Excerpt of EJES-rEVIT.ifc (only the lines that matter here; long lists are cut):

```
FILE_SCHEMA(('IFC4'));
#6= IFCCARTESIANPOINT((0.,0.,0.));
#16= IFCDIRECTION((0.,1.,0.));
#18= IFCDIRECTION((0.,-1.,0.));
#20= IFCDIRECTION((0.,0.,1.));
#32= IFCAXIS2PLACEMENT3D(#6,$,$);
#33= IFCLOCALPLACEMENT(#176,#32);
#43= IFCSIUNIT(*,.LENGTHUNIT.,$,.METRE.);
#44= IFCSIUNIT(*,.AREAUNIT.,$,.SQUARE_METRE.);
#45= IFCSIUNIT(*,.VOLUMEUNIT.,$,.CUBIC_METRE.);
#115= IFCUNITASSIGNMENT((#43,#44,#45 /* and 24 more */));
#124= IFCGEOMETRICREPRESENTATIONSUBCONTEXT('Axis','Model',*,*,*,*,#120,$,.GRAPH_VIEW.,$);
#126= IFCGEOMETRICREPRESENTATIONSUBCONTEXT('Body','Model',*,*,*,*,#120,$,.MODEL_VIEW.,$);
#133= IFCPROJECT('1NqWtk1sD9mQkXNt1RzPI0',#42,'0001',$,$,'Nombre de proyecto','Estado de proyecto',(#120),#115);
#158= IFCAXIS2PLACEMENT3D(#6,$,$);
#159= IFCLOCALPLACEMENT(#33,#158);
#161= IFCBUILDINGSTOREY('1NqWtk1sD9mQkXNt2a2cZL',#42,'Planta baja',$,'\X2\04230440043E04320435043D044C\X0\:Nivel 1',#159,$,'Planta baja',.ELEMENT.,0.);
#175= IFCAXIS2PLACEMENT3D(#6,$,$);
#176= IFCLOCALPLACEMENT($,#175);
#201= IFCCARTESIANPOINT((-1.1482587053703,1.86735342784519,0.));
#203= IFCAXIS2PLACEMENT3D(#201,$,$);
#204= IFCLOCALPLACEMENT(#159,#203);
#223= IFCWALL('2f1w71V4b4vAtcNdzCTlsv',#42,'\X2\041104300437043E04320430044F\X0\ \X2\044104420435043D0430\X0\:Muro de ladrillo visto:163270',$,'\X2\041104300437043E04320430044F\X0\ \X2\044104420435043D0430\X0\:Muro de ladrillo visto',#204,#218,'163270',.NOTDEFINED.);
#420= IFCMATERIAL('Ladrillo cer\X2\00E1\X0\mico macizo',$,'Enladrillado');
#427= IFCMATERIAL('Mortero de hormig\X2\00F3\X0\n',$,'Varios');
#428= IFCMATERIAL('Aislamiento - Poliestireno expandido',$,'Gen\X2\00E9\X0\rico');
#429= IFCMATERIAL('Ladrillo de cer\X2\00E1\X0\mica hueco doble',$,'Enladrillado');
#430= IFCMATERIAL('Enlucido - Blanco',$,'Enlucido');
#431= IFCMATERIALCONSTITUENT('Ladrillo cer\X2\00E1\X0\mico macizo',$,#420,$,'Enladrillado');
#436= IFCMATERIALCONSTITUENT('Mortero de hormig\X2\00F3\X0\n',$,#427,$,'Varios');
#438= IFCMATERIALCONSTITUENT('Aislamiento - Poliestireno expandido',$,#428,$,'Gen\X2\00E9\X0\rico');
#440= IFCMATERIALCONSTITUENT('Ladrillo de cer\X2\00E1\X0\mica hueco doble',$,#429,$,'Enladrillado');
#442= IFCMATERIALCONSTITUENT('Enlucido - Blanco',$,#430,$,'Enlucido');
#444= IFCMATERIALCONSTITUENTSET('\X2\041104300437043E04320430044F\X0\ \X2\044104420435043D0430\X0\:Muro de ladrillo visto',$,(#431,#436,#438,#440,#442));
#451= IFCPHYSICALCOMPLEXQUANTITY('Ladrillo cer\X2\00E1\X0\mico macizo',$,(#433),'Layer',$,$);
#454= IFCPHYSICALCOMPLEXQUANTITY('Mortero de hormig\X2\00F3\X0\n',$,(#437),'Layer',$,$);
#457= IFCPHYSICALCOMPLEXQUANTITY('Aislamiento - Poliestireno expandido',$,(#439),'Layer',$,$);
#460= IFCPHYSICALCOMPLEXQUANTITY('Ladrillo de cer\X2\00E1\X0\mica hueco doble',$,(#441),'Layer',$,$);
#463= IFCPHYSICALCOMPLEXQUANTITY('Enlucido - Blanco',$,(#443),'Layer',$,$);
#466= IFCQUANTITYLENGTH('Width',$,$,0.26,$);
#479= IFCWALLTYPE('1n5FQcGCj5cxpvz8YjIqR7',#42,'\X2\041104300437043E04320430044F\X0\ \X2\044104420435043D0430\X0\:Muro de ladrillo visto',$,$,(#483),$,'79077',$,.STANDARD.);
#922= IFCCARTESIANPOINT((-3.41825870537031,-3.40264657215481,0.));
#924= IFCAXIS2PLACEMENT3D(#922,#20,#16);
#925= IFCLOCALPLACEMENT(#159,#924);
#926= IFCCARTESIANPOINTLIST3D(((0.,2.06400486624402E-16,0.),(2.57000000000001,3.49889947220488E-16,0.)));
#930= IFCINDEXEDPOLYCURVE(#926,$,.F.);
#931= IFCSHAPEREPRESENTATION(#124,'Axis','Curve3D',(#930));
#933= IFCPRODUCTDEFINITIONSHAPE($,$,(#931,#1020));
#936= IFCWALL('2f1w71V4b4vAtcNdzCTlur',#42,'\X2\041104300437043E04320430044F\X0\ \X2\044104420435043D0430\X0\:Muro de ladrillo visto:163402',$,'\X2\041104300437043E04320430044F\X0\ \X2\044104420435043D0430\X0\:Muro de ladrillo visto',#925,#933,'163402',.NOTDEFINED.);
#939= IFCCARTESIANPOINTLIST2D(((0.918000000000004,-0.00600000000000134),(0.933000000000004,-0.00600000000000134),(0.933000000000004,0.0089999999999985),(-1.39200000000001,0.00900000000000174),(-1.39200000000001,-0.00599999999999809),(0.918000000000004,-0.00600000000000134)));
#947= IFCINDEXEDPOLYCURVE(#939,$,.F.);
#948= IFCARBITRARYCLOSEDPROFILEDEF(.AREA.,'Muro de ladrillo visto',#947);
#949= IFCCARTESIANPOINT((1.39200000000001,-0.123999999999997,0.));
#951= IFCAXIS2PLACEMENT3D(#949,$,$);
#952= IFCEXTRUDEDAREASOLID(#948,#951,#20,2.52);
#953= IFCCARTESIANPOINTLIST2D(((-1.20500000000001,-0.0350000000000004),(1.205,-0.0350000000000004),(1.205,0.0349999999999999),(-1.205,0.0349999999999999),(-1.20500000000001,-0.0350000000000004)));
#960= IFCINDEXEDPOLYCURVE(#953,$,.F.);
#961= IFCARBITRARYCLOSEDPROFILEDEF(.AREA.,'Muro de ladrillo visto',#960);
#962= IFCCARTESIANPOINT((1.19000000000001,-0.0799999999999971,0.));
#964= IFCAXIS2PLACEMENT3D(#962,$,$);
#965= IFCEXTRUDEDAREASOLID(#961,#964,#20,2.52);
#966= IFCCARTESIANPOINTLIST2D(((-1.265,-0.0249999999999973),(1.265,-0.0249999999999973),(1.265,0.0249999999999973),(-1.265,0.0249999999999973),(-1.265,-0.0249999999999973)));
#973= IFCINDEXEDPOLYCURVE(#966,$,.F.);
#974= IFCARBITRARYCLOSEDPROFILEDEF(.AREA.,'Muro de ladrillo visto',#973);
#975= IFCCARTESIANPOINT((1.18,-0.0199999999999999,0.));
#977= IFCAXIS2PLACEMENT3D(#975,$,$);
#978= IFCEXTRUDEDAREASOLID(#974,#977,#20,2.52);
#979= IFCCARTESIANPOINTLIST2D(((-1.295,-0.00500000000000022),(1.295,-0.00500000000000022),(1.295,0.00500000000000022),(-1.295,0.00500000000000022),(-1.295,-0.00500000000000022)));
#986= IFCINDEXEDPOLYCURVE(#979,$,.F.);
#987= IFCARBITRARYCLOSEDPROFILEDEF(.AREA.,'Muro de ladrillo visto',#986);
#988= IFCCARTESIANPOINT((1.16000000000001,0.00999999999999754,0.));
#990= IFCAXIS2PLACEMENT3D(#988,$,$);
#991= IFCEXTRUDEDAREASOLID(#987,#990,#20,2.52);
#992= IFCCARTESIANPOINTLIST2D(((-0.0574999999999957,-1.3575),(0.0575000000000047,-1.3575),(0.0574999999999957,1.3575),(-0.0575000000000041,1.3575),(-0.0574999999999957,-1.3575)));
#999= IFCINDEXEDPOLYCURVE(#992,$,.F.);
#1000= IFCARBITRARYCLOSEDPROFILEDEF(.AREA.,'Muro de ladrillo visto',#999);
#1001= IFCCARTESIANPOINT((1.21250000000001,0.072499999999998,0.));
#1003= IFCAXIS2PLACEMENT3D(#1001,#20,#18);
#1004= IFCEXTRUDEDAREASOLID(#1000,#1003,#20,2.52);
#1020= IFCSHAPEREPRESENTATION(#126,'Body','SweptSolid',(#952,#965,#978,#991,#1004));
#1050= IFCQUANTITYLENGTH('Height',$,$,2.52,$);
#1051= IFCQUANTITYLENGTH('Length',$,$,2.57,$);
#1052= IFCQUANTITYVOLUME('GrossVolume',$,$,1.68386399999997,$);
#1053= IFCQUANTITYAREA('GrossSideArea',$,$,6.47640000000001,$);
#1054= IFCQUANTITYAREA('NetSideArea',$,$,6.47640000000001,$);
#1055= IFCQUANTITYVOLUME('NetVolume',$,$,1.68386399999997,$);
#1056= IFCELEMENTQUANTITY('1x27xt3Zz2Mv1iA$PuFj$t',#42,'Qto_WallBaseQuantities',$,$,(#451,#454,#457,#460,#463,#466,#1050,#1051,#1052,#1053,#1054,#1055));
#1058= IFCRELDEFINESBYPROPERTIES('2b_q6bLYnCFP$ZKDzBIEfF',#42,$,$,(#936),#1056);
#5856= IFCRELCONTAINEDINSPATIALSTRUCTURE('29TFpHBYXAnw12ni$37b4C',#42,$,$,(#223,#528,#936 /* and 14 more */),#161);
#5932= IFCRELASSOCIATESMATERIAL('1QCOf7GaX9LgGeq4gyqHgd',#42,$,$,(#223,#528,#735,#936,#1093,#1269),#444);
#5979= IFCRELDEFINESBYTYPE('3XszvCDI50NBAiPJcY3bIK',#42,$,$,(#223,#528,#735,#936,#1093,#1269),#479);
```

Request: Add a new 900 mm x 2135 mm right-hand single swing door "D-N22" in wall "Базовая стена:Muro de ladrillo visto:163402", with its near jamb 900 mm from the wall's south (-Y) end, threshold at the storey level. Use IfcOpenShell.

```python
import numpy as np
import ifcopenshell
import ifcopenshell.api.feature
import ifcopenshell.api.geometry
import ifcopenshell.api.pset
import ifcopenshell.api.root
import ifcopenshell.api.spatial
import ifcopenshell.geom
import ifcopenshell.util.element
import ifcopenshell.util.placement
import ifcopenshell.util.representation
import ifcopenshell.util.shape
import ifcopenshell.util.unit

model = ifcopenshell.open("EJES-rEVIT.ifc")
unit_scale = ifcopenshell.util.unit.calculate_unit_scale(model)
area_scale = ifcopenshell.util.unit.calculate_unit_scale(model, "AREAUNIT")
volume_scale = ifcopenshell.util.unit.calculate_unit_scale(model, "VOLUMEUNIT")
settings = ifcopenshell.geom.settings()


def volume(element):
    """Net volume in cubic metres, openings subtracted."""
    shape = ifcopenshell.geom.create_shape(settings, element)
    return ifcopenshell.util.shape.get_volume(shape.geometry)


wall = model.by_guid("2f1w71V4b4vAtcNdzCTlur")
storey = ifcopenshell.util.element.get_container(wall, ifc_class="IfcBuildingStorey")
context = ifcopenshell.util.representation.get_context(model, "Model", "Body", "MODEL_VIEW")
before = volume(wall)

width, height, from_end, sill = 0.9, 2.135, 0.9, 0.0  # metres

# The wall runs along its own X axis, and the end named is its -X end.
wall_shape = ifcopenshell.geom.create_shape(settings, wall)
x, y, z = ifcopenshell.util.shape.get_vertices(wall_shape.geometry).T
start = x.min() + from_end
face, thickness = float(y.min()), float(y.max() - y.min())
wall_matrix = ifcopenshell.util.placement.get_local_placement(wall.ObjectPlacement)
level = ifcopenshell.util.placement.get_local_placement(storey.ObjectPlacement)[2, 3]


def in_wall(x, y):
    """Placement at x, y metres in the wall's axes, at sill height."""
    matrix = wall_matrix.copy()
    matrix[:, 3] = wall_matrix @ np.array([x / unit_scale, y / unit_scale, 0.0, 1.0])
    matrix[2, 3] = level + sill / unit_scale
    return matrix


# Opening: a box that overshoots both wall faces by 50 mm.
opening = ifcopenshell.api.root.create_entity(model, ifc_class="IfcOpeningElement", predefined_type="OPENING")
box = ifcopenshell.api.geometry.add_wall_representation(
    model, context=context, length=width, height=height, thickness=thickness + 0.1
)
ifcopenshell.api.geometry.assign_representation(model, product=opening, representation=box)
ifcopenshell.api.geometry.edit_object_placement(model, product=opening, matrix=in_wall(start, face - 0.05), is_si=False)
ifcopenshell.api.feature.add_feature(model, feature=opening, element=wall)

door = ifcopenshell.api.root.create_entity(model, ifc_class="IfcDoor", name="D-N22", predefined_type="DOOR")
door.OverallWidth, door.OverallHeight = width / unit_scale, height / unit_scale
door.OperationType = "SINGLE_SWING_RIGHT"
body = ifcopenshell.api.geometry.add_door_representation(
    model,
    context=context,
    overall_width=door.OverallWidth,
    overall_height=door.OverallHeight,
    operation_type="SINGLE_SWING_RIGHT",
    lining_properties={"LiningDepth": thickness / unit_scale, "ThresholdDepth": thickness / unit_scale},
)
ifcopenshell.api.geometry.assign_representation(model, product=door, representation=body)
ifcopenshell.api.spatial.assign_container(model, products=[door], relating_structure=storey)
ifcopenshell.api.feature.add_filling(model, opening=opening, element=door)

# The lining spans the wall, so the door starts at the wall face.
ifcopenshell.api.geometry.edit_object_placement(model, product=door, matrix=in_wall(start, face), is_si=False)

after = volume(wall)

# Update the wall's stored quantities.
qto = model.by_id(ifcopenshell.util.element.get_pset(wall, "Qto_WallBaseQuantities", should_inherit=False)["id"])
ifcopenshell.api.pset.edit_qto(model, qto=qto, properties={
    "NetSideArea": after / thickness / area_scale,
    "NetVolume": after / volume_scale,
})

print(f"wall volume {before:.3f} -> {after:.3f} m3")

model.write("EJES-rEVIT_updated.ifc")
```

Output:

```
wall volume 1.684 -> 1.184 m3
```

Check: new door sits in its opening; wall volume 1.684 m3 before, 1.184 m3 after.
